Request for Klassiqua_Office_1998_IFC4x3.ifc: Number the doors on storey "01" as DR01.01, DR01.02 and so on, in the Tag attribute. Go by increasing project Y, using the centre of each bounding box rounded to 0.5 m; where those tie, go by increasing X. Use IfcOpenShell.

First a look at what the model holds.

```python
import ifcopenshell
import ifcopenshell.util.element
import ifcopenshell.util.placement

model = ifcopenshell.open("Klassiqua_Office_1998_IFC4x3.ifc")
print(model.schema)
storey = next(s for s in model.by_type("IfcBuildingStorey") if s.Name == "01")
doors = [e for e in ifcopenshell.util.element.get_decomposition(storey) if e.is_a("IfcDoor")]
for e in sorted(doors, key=lambda e: e.id()):
    origin = ifcopenshell.util.placement.get_local_placement(e.ObjectPlacement)[:3, 3]
    print(e.id(), e.Tag, e.Name, origin.round(2) + 0.0, sep=" | ")
```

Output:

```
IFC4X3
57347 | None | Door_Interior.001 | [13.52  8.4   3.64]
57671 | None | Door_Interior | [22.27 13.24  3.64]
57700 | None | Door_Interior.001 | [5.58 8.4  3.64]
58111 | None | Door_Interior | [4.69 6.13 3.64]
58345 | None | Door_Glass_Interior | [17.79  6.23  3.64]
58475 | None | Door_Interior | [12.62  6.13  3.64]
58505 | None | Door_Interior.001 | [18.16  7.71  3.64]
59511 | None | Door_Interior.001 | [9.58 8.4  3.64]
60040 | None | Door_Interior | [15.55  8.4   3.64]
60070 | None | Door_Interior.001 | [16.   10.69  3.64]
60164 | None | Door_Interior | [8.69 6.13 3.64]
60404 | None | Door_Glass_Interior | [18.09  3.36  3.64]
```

```python
import ifcopenshell
import ifcopenshell.geom
import ifcopenshell.util.element
import ifcopenshell.util.shape

model = ifcopenshell.open("Klassiqua_Office_1998_IFC4x3.ifc")
settings = ifcopenshell.geom.settings()
settings.set("use-world-coords", True)


def centre(element):
    shape = ifcopenshell.geom.create_shape(settings, element)
    return ifcopenshell.util.shape.get_bbox_centroid(shape.geometry)


storey = next(s for s in model.by_type("IfcBuildingStorey") if s.Name == "01")
doors = [e for e in ifcopenshell.util.element.get_decomposition(storey) if e.is_a("IfcDoor")]

# Insertion points can sit at a corner or the storey origin, so sort by the geometry (in metres).
centres = {e: centre(e) for e in doors}
doors.sort(key=lambda e: (round(centres[e][1] / 0.5), centres[e][0]))

for i, e in enumerate(doors, start=1):
    number = f"DR01.{i:02d}"
    e.Tag = number
    print(e.id(), number)

model.write("Klassiqua_Office_1998_IFC4x3_v2.ifc")
```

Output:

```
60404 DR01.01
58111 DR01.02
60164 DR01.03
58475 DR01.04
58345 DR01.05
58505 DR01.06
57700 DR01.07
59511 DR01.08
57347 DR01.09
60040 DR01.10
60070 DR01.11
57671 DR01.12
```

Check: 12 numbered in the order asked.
